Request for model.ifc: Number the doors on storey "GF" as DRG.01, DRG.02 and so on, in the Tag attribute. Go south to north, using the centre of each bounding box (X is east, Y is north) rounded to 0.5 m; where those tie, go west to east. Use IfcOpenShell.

First a look at what the model holds.

```python
import ifcopenshell
import ifcopenshell.util.element
import ifcopenshell.util.placement

model = ifcopenshell.open("model.ifc")
print(model.schema)
storey = next(s for s in model.by_type("IfcBuildingStorey") if s.Name == "GF")
doors = [e for e in ifcopenshell.util.element.get_decomposition(storey) if e.is_a("IfcDoor")]
for e in sorted(doors, key=lambda e: e.id()):
    origin = ifcopenshell.util.placement.get_local_placement(e.ObjectPlacement)[:3, 3]
    print(e.id(), e.Tag, e.Name, origin.round(2) + 0.0, sep=" | ")
```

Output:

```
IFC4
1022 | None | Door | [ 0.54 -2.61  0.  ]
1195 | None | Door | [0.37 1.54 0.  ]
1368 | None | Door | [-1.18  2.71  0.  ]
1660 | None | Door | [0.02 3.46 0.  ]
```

```python
import ifcopenshell
import ifcopenshell.geom
import ifcopenshell.util.element
import ifcopenshell.util.shape

model = ifcopenshell.open("model.ifc")
settings = ifcopenshell.geom.settings()
settings.set("use-world-coords", True)


def centre(element):
    shape = ifcopenshell.geom.create_shape(settings, element)
    return ifcopenshell.util.shape.get_bbox_centroid(shape.geometry)


storey = next(s for s in model.by_type("IfcBuildingStorey") if s.Name == "GF")
doors = [e for e in ifcopenshell.util.element.get_decomposition(storey) if e.is_a("IfcDoor")]

# Insertion points can sit at a corner or the storey origin, so sort by the geometry (in metres).
centres = {e: centre(e) for e in doors}
doors.sort(key=lambda e: (round(centres[e][1] / 0.5), centres[e][0]))

for i, e in enumerate(doors, start=1):
    number = f"DRG.{i:02d}"
    e.Tag = number
    print(e.id(), number)

model.write("model_updated.ifc")
```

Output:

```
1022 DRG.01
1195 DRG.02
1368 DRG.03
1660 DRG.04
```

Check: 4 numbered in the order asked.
